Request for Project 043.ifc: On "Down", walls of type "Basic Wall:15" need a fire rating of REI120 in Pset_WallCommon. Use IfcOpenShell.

First a look at what the model holds.

```python
import ifcopenshell
import ifcopenshell.util.element

model = ifcopenshell.open("Project 043.ifc")
print(model.schema)
storey = next(s for s in model.by_type("IfcBuildingStorey") if s.Name == "Down")
walls = [e for e in ifcopenshell.util.element.get_decomposition(storey) if e.is_a("IfcWall")]
seen = {}
for e in walls:
    element_type = ifcopenshell.util.element.get_type(e)
    key = (element_type.Name if element_type != e and element_type else None, ifcopenshell.util.element.get_pset(e, "Pset_WallCommon", "FireRating"))
    seen[key] = seen.get(key, 0) + 1
for (name, value), count in sorted(seen.items(), key=str):
    print(count, "x", name, "|", value)
```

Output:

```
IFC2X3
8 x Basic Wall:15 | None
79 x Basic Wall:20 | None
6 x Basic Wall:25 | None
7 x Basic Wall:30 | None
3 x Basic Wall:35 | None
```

```python
import ifcopenshell
import ifcopenshell.api.pset
import ifcopenshell.util.element

model = ifcopenshell.open("Project 043.ifc")

storey = next(s for s in model.by_type("IfcBuildingStorey") if s.Name == "Down")
walls = [e for e in ifcopenshell.util.element.get_decomposition(storey) if e.is_a("IfcWall")]

count = 0
for e in walls:
    element_type = ifcopenshell.util.element.get_type(e)
    if element_type in (None, e) or element_type.Name != "Basic Wall:15":
        continue
    # add_pset returns the element's existing set when there is one.
    pset = ifcopenshell.api.pset.add_pset(model, product=e, name="Pset_WallCommon")
    ifcopenshell.api.pset.edit_pset(model, pset=pset, properties={"FireRating": "REI120"})
    count += 1

print(count, "walls updated")

model.write("Project 043-out.ifc")
```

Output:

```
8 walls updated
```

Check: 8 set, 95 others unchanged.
